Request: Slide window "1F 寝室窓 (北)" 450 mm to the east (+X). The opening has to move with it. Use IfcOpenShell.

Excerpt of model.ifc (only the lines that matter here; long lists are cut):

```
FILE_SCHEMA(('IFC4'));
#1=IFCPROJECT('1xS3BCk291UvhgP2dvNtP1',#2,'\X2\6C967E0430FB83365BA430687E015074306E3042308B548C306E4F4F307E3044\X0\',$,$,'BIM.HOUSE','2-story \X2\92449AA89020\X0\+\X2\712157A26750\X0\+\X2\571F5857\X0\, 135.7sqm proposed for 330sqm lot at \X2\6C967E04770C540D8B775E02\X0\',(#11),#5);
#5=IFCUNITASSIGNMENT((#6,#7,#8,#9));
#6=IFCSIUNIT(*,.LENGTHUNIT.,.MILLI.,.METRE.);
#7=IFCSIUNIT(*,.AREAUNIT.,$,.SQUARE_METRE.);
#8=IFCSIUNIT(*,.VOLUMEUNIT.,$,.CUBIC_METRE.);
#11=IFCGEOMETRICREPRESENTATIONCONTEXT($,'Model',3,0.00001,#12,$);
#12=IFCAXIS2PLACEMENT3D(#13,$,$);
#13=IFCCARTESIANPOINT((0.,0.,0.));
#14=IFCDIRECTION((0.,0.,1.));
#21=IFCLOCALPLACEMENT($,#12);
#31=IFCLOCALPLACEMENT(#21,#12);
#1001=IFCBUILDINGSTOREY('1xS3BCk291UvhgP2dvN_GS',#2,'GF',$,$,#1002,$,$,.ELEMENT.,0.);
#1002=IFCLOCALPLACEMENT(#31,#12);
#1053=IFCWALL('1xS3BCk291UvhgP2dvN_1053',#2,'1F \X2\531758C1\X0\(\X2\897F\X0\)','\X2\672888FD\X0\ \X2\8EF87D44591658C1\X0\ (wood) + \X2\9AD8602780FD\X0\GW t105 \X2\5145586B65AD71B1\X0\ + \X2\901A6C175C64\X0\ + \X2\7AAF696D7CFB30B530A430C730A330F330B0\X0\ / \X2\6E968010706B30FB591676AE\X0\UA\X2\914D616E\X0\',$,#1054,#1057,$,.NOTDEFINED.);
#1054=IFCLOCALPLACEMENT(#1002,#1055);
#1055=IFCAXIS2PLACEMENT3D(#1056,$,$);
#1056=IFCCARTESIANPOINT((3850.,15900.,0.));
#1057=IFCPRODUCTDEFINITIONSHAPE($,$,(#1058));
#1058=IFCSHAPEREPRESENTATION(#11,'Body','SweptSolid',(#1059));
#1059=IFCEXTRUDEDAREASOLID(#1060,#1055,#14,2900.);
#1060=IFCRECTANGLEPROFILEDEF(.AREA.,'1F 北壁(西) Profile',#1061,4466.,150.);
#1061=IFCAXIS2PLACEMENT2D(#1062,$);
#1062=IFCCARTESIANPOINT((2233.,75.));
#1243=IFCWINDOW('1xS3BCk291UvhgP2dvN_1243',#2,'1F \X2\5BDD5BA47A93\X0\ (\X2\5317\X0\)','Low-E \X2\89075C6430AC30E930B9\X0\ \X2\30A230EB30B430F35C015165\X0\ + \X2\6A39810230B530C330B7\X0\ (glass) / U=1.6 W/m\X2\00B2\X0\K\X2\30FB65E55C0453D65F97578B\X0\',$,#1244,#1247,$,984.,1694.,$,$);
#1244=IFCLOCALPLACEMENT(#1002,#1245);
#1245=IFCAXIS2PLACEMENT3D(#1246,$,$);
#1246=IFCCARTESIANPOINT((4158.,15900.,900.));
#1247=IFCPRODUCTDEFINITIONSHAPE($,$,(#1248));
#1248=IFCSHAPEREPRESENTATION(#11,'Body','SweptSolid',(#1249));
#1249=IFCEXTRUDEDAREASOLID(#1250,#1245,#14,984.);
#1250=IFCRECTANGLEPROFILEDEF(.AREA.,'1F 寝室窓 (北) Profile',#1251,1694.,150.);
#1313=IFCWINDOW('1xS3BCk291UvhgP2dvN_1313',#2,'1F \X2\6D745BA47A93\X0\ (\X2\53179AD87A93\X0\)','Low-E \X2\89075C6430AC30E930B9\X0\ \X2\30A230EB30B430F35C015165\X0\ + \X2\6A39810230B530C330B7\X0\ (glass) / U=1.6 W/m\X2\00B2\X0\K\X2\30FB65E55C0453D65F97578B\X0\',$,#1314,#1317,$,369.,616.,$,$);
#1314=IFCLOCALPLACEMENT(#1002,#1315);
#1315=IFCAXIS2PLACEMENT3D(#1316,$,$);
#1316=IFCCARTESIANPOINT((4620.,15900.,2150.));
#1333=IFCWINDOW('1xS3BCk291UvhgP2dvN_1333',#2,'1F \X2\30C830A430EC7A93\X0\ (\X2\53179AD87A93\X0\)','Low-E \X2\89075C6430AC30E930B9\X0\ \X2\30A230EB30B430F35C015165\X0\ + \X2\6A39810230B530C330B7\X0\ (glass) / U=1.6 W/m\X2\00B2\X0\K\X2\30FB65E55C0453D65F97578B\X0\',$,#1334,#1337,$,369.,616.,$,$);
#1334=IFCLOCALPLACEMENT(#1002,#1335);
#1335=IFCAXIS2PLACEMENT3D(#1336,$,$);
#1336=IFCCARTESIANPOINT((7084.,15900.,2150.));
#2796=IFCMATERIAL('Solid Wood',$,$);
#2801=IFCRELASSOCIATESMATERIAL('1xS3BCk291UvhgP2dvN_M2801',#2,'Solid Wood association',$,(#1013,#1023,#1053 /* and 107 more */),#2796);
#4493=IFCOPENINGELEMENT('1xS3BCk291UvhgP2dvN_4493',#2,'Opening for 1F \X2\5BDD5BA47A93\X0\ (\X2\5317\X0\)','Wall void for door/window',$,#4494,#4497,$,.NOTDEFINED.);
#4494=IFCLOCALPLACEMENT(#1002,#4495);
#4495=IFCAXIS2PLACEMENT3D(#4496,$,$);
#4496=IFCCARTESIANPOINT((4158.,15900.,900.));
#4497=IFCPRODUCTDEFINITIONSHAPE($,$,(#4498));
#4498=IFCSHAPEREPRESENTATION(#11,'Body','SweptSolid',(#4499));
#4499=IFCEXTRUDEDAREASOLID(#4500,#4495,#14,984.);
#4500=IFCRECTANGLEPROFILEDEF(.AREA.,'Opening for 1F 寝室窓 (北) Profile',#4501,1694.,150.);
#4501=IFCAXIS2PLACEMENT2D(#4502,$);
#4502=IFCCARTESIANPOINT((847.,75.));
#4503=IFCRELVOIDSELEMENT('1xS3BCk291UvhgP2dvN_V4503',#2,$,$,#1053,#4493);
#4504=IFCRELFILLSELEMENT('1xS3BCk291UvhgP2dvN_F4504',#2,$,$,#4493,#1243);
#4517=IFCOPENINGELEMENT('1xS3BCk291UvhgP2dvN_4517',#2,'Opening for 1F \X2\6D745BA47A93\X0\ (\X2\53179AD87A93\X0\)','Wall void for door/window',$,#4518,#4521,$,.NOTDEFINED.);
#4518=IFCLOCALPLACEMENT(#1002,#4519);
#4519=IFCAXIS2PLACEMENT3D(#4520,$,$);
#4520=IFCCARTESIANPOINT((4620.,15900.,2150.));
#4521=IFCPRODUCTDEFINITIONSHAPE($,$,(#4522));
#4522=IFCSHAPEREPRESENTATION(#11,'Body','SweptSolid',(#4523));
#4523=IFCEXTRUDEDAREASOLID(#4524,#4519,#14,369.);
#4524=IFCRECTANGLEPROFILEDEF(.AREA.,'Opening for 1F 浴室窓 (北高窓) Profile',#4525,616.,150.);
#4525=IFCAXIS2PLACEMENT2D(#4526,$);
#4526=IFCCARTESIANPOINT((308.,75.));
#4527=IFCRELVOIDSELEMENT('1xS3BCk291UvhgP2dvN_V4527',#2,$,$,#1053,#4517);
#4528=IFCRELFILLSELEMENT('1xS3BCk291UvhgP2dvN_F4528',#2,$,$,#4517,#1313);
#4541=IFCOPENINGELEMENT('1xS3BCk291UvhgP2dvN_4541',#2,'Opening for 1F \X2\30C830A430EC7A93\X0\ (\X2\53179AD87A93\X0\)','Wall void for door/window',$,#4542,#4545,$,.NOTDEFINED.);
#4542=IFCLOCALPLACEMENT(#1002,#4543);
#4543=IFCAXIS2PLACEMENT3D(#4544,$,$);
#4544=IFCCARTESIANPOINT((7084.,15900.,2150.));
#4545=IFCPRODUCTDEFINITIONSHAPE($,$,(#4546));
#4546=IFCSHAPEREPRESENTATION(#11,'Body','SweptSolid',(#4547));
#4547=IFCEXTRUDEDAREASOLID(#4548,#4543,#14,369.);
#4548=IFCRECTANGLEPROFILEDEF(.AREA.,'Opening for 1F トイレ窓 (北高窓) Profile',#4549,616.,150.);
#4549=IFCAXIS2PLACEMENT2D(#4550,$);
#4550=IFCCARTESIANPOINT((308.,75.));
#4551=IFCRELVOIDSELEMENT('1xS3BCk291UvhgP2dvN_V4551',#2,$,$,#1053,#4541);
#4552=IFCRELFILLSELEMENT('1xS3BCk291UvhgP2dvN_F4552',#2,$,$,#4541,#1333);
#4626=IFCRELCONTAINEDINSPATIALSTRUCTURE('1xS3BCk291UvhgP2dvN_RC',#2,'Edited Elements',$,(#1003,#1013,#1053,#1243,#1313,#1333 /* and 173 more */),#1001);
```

```python
import ifcopenshell
import ifcopenshell.api.geometry
import ifcopenshell.util.placement

model = ifcopenshell.open("model.ifc")

window = model.by_id(1243)
opening = window.FillsVoids[0].RelatingOpeningElement
wall = opening.VoidsElements[0].RelatingBuildingElement

wall_matrix = ifcopenshell.util.placement.get_local_placement(wall.ObjectPlacement)
shift = wall_matrix[:3, 0] * 450.0
before = ifcopenshell.util.placement.get_local_placement(window.ObjectPlacement)[:3, 3].copy()

# The window is not placed relative to its opening, so move both.
for product in (opening, window):
    matrix = ifcopenshell.util.placement.get_local_placement(product.ObjectPlacement)
    matrix[:3, 3] += shift
    ifcopenshell.api.geometry.edit_object_placement(model, product=product, matrix=matrix, is_si=False)

after = ifcopenshell.util.placement.get_local_placement(window.ObjectPlacement)[:3, 3]
print("window moved by", (after - before).round(3) + 0.0)

model.write("model-out.ifc")
```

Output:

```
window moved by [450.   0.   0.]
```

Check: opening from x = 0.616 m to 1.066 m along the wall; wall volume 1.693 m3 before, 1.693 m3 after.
